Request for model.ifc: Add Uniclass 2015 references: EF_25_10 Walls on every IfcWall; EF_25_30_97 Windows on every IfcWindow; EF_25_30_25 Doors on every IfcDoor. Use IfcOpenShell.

First a look at what the model holds.

```python
import ifcopenshell

model = ifcopenshell.open("model.ifc")
print(model.schema)
print("classifications:", [c.Name for c in model.by_type("IfcClassification")])
for ifc_class in ("IfcDoor", "IfcRoof", "IfcStair", "IfcWall", "IfcWindow"):
    print(ifc_class, len(model.by_type(ifc_class)))
```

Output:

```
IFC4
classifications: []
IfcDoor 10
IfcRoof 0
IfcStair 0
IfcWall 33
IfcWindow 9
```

```python
import ifcopenshell
import ifcopenshell.api.classification

model = ifcopenshell.open("model.ifc")

system = ifcopenshell.api.classification.add_classification(model, classification="Uniclass 2015")

codes = {
    "IfcWall": ("EF_25_10", "Walls"),
    "IfcWindow": ("EF_25_30_97", "Windows"),
    "IfcDoor": ("EF_25_30_25", "Doors"),
}
for ifc_class, (code, name) in codes.items():
    products = model.by_type(ifc_class)
    ifcopenshell.api.classification.add_reference(
        model, products=products, classification=system, identification=code, name=name
    )
    print(code, len(products))

model.write("model_v2.ifc")
```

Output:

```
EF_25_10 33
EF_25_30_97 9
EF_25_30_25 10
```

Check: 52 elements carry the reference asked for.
